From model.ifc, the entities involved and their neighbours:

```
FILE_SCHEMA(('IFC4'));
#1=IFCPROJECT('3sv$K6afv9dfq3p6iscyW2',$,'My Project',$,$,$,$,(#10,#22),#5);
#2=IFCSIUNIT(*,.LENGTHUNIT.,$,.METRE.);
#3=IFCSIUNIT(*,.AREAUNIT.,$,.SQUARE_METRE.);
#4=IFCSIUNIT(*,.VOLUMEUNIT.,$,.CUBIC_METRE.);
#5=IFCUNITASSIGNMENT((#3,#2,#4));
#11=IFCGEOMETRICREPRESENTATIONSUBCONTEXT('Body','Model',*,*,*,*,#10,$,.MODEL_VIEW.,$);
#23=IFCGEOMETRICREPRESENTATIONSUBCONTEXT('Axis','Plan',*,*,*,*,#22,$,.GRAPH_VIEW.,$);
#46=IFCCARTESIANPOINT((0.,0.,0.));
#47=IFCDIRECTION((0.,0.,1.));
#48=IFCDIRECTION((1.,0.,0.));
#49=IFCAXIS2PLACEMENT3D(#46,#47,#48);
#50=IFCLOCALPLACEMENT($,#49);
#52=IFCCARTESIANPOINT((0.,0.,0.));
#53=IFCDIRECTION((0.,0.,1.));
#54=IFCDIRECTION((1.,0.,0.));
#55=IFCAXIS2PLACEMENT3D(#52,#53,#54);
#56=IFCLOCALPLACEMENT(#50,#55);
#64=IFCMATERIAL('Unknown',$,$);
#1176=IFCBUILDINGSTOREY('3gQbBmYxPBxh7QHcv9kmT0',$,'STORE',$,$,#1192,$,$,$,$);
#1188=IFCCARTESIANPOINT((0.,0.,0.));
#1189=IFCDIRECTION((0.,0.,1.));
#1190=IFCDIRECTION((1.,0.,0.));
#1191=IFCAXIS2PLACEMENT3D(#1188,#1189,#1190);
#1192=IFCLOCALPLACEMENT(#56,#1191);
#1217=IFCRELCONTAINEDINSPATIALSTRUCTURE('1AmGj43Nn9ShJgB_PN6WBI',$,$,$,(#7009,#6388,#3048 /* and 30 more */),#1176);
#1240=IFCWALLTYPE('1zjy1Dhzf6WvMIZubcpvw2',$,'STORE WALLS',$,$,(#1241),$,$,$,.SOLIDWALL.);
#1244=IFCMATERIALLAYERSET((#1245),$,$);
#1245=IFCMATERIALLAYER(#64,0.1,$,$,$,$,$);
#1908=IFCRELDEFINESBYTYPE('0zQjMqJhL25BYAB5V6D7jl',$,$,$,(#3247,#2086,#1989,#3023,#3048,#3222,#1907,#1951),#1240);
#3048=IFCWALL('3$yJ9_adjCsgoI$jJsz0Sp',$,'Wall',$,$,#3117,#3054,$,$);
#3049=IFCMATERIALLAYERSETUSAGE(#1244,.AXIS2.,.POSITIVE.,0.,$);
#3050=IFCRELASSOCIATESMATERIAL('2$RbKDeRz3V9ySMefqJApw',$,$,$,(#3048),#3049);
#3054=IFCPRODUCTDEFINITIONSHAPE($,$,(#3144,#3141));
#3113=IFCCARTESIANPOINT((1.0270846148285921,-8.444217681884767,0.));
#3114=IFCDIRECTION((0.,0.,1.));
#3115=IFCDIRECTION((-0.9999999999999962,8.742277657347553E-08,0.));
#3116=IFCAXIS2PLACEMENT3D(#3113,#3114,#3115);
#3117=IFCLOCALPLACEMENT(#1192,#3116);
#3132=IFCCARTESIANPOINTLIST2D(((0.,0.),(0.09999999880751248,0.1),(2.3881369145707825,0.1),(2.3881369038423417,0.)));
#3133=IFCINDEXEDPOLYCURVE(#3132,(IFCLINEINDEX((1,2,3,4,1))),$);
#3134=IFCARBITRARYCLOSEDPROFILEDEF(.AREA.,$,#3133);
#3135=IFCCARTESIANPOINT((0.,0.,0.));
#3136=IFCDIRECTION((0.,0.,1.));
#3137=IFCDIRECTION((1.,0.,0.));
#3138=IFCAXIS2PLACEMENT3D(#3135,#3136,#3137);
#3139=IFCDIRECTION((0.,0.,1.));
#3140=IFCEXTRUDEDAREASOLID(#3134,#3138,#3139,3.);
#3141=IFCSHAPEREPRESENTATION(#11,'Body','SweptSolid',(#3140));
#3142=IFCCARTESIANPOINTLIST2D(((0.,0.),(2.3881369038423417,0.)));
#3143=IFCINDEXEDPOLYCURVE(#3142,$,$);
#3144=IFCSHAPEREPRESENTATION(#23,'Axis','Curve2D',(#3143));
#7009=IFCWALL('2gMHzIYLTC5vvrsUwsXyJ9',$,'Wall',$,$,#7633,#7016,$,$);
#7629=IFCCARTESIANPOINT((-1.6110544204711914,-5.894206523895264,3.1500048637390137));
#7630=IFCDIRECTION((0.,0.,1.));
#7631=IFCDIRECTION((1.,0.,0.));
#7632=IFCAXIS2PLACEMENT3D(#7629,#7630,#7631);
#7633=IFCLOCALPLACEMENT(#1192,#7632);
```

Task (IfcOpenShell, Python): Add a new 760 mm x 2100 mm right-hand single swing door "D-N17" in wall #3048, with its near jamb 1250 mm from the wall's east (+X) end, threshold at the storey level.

```python
import numpy as np
import ifcopenshell
import ifcopenshell.api.feature
import ifcopenshell.api.geometry
import ifcopenshell.api.root
import ifcopenshell.api.spatial
import ifcopenshell.geom
import ifcopenshell.util.element
import ifcopenshell.util.placement
import ifcopenshell.util.representation
import ifcopenshell.util.shape
import ifcopenshell.util.unit

model = ifcopenshell.open("model.ifc")
unit_scale = ifcopenshell.util.unit.calculate_unit_scale(model)
settings = ifcopenshell.geom.settings()


def volume(element):
    """Net volume in cubic metres, openings subtracted."""
    shape = ifcopenshell.geom.create_shape(settings, element)
    return ifcopenshell.util.shape.get_volume(shape.geometry)


wall = model.by_id(3048)
storey = ifcopenshell.util.element.get_container(wall, ifc_class="IfcBuildingStorey")
context = ifcopenshell.util.representation.get_context(model, "Model", "Body", "MODEL_VIEW")
before = volume(wall)

width, height, from_end, sill = 0.76, 2.1, 1.25, 0.0  # metres

# The wall runs along its own X axis, and the end named is its -X end.
wall_shape = ifcopenshell.geom.create_shape(settings, wall)
x, y, z = ifcopenshell.util.shape.get_vertices(wall_shape.geometry).T
start = x.min() + from_end
face, thickness = float(y.min()), float(y.max() - y.min())
wall_matrix = ifcopenshell.util.placement.get_local_placement(wall.ObjectPlacement)
level = ifcopenshell.util.placement.get_local_placement(storey.ObjectPlacement)[2, 3]


def in_wall(x, y):
    """Placement at x, y metres in the wall's axes, at sill height."""
    matrix = wall_matrix.copy()
    matrix[:, 3] = wall_matrix @ np.array([x / unit_scale, y / unit_scale, 0.0, 1.0])
    matrix[2, 3] = level + sill / unit_scale
    return matrix


# Opening: a box that overshoots both wall faces by 50 mm.
opening = ifcopenshell.api.root.create_entity(model, ifc_class="IfcOpeningElement", predefined_type="OPENING")
box = ifcopenshell.api.geometry.add_wall_representation(
    model, context=context, length=width, height=height, thickness=thickness + 0.1
)
ifcopenshell.api.geometry.assign_representation(model, product=opening, representation=box)
ifcopenshell.api.geometry.edit_object_placement(model, product=opening, matrix=in_wall(start, face - 0.05), is_si=False)
ifcopenshell.api.feature.add_feature(model, feature=opening, element=wall)

door = ifcopenshell.api.root.create_entity(model, ifc_class="IfcDoor", name="D-N17", predefined_type="DOOR")
door.OverallWidth, door.OverallHeight = width / unit_scale, height / unit_scale
door.OperationType = "SINGLE_SWING_RIGHT"
body = ifcopenshell.api.geometry.add_door_representation(
    model,
    context=context,
    overall_width=door.OverallWidth,
    overall_height=door.OverallHeight,
    operation_type="SINGLE_SWING_RIGHT",
    lining_properties={"LiningDepth": thickness / unit_scale, "ThresholdDepth": thickness / unit_scale},
)
ifcopenshell.api.geometry.assign_representation(model, product=door, representation=body)
ifcopenshell.api.spatial.assign_container(model, products=[door], relating_structure=storey)
ifcopenshell.api.feature.add_filling(model, opening=opening, element=door)

# The lining spans the wall, so the door starts at the wall face.
ifcopenshell.api.geometry.edit_object_placement(model, product=door, matrix=in_wall(start, face), is_si=False)

after = volume(wall)

print(f"wall volume {before:.3f} -> {after:.3f} m3")

model.write("model_rev.ifc")
```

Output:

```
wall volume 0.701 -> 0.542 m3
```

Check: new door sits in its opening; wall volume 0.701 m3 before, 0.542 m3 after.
